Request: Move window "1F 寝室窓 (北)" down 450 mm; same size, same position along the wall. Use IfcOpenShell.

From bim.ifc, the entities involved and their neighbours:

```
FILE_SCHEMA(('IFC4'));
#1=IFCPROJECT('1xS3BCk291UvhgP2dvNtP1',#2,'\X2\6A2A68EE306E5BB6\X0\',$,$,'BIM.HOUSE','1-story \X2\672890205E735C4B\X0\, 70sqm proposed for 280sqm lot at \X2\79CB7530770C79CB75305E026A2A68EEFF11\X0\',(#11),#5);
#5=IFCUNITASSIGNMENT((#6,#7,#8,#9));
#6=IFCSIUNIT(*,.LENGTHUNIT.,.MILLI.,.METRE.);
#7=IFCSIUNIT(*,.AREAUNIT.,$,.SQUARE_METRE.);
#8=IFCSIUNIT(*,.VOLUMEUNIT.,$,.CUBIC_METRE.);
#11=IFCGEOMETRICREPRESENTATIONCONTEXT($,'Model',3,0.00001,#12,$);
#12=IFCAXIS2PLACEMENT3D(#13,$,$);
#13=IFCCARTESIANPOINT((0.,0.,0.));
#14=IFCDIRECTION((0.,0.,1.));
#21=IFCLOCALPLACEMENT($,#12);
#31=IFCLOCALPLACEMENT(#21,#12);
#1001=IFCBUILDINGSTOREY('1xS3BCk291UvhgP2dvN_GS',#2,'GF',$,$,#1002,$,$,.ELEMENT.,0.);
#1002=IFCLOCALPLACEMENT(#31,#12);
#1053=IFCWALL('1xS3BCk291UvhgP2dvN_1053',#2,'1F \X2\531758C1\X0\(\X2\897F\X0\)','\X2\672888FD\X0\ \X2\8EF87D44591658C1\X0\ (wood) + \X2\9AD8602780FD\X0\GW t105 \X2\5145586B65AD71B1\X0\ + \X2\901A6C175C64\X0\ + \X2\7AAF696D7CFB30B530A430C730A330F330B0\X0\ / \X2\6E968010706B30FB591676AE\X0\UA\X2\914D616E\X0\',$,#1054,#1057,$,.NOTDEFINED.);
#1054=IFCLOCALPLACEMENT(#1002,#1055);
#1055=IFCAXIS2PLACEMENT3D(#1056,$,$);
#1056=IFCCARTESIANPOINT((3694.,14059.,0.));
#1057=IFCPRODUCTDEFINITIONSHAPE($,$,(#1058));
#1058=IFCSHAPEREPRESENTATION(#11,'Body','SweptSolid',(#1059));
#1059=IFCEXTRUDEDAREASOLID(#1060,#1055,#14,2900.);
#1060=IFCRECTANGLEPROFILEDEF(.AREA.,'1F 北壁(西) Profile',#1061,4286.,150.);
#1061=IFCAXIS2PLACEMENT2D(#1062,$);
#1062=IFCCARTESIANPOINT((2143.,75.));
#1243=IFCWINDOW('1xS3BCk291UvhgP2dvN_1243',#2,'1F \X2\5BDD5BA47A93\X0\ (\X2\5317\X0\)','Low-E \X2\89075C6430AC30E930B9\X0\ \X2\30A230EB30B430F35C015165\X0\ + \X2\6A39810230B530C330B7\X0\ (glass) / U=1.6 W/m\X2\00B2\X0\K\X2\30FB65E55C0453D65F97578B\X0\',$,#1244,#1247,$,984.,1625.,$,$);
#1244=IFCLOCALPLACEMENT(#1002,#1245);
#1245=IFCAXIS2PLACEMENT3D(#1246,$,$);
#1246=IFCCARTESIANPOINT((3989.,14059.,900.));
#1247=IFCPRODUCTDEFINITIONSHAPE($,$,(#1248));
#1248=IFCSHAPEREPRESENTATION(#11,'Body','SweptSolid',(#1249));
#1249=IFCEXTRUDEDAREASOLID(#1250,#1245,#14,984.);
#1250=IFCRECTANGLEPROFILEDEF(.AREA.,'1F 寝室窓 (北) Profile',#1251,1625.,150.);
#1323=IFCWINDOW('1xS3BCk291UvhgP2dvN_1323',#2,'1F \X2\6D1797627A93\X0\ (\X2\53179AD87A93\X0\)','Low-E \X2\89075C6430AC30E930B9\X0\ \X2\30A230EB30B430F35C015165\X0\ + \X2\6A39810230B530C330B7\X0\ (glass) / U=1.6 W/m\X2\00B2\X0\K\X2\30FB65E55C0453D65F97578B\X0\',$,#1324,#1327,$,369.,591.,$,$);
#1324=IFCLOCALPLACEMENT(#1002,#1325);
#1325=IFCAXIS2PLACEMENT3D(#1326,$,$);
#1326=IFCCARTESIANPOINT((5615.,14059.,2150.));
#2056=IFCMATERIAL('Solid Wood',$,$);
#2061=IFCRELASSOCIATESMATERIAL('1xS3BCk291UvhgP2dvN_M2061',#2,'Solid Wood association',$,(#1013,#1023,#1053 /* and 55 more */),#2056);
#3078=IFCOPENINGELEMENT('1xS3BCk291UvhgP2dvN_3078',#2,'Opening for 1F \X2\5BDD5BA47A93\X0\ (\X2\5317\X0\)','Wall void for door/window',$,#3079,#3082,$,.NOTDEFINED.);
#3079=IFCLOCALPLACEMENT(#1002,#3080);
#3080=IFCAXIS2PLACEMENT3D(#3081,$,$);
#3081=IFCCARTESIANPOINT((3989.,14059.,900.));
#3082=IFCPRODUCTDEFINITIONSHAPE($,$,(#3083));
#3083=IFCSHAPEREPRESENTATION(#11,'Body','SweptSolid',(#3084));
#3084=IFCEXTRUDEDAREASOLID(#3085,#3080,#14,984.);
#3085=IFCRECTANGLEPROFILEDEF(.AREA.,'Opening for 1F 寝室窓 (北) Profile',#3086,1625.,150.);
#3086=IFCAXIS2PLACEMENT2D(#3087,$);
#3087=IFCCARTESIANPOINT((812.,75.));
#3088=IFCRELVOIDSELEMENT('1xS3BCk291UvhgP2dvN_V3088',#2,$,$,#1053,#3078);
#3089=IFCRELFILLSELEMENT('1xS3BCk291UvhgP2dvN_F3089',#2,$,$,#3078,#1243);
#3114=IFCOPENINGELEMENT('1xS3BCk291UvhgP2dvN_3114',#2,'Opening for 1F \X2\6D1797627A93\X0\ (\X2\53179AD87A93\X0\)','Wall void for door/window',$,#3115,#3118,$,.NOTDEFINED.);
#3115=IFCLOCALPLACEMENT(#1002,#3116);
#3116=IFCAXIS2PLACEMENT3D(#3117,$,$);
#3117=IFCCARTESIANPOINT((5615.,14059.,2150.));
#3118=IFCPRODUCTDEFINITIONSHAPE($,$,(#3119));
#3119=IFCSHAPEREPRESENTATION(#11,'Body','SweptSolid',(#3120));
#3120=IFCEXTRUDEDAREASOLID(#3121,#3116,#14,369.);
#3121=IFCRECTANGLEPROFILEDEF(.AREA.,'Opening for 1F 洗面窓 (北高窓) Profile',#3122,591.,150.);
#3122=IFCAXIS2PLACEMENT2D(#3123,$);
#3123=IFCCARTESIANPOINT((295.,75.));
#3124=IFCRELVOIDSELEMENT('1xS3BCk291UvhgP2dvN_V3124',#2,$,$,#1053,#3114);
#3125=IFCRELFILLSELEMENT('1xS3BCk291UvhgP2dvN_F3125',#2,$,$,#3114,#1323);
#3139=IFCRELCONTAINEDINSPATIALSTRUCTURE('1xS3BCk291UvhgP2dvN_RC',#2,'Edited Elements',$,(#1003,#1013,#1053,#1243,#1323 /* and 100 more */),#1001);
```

```python
import numpy as np
import ifcopenshell
import ifcopenshell.api.geometry
import ifcopenshell.util.placement
import ifcopenshell.util.unit

model = ifcopenshell.open("bim.ifc")
unit_scale = ifcopenshell.util.unit.calculate_unit_scale(model)

window = model.by_guid("1xS3BCk291UvhgP2dvN_1243")
opening = window.FillsVoids[0].RelatingOpeningElement
dz = -0.45 / unit_scale

shift = np.array([0.0, 0.0, dz])
# The window is not placed relative to its opening, so move both.
for product in (opening, window):
    matrix = ifcopenshell.util.placement.get_local_placement(product.ObjectPlacement)
    matrix[:3, 3] += shift
    ifcopenshell.api.geometry.edit_object_placement(model, product=product, matrix=matrix, is_si=False)

print(f"moved by {dz * unit_scale:+.3f} m")

model.write("bim-out.ifc")
```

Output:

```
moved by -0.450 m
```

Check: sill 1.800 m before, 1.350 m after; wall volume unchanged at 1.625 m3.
